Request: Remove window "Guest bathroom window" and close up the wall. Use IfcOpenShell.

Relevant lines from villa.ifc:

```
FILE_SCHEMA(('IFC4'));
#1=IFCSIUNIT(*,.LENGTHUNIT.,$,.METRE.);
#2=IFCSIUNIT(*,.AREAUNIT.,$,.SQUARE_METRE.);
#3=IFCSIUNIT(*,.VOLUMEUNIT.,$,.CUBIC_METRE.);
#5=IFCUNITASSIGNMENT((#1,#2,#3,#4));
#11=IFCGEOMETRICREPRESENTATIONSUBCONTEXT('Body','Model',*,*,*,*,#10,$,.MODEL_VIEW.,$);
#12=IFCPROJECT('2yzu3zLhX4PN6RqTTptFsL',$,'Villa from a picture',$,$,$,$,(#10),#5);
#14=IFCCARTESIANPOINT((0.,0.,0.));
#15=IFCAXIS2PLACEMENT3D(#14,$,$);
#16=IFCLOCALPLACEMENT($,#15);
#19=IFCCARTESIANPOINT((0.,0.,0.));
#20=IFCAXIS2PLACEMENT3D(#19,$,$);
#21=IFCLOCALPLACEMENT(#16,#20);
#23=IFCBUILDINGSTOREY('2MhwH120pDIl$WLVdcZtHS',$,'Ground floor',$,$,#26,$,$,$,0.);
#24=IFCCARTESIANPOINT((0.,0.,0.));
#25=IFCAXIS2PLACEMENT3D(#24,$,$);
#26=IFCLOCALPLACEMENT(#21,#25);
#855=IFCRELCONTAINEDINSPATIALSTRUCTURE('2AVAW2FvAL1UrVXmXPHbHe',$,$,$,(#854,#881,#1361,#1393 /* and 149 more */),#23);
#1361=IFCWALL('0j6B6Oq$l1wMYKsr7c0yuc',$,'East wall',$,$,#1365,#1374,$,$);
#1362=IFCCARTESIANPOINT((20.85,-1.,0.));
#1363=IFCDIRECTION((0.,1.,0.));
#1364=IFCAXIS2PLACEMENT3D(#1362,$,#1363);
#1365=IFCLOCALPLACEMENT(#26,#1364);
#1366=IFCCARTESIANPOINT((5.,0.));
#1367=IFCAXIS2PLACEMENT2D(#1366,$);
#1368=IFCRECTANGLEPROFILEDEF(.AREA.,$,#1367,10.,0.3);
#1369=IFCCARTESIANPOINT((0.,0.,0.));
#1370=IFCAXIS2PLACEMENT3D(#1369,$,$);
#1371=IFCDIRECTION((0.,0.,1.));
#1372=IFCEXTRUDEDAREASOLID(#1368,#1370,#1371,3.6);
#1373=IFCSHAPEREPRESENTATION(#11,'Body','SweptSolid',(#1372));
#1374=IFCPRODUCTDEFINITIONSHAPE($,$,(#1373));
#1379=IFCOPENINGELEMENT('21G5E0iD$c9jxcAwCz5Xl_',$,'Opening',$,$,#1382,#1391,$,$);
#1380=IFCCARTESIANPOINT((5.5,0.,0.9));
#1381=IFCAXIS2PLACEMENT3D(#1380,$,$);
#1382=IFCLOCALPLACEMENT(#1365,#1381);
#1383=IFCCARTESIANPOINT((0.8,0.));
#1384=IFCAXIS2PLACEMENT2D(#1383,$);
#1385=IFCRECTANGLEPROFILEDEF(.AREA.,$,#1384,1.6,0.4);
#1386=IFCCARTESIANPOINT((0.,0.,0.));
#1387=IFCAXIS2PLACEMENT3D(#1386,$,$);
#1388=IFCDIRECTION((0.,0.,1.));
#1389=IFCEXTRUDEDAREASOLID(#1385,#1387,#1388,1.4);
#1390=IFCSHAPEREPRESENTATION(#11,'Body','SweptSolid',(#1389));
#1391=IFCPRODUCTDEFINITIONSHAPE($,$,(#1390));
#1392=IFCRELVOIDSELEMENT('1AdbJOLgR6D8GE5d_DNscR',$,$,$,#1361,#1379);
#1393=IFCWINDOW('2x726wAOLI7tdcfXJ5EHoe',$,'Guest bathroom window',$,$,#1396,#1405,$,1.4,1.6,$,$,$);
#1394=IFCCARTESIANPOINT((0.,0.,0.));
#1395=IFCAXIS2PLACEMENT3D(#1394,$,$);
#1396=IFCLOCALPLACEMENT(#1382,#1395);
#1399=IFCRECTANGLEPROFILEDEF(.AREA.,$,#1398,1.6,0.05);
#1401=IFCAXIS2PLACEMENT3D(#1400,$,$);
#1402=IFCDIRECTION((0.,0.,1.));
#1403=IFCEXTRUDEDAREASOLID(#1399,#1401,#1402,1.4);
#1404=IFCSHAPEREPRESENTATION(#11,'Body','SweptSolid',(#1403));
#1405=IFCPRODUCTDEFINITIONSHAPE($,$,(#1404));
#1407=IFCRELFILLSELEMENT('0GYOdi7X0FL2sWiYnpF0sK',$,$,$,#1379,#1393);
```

```python
import ifcopenshell
import ifcopenshell.api.feature
import ifcopenshell.api.root
import ifcopenshell.geom
import ifcopenshell.util.shape

model = ifcopenshell.open("villa.ifc")
settings = ifcopenshell.geom.settings()


def volume(element):
    """Net volume in cubic metres, openings subtracted."""
    shape = ifcopenshell.geom.create_shape(settings, element)
    return ifcopenshell.util.shape.get_volume(shape.geometry)


window = model.by_guid("2x726wAOLI7tdcfXJ5EHoe")
opening = window.FillsVoids[0].RelatingOpeningElement
wall = opening.VoidsElements[0].RelatingBuildingElement
before = volume(wall)

ifcopenshell.api.root.remove_product(model, product=window)
ifcopenshell.api.feature.remove_feature(model, feature=opening)

after = volume(wall)

print(f"wall volume {before:.3f} -> {after:.3f} m3")

model.write("villa_v2.ifc")
```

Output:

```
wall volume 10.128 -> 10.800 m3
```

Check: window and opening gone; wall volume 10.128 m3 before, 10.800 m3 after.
